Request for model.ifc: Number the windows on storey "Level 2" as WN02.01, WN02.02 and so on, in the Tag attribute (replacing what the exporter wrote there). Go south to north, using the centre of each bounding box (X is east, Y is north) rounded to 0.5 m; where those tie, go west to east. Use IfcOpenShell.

First a look at what the model holds.

```python
import ifcopenshell
import ifcopenshell.util.element
import ifcopenshell.util.placement

model = ifcopenshell.open("model.ifc")
print(model.schema)
storey = next(s for s in model.by_type("IfcBuildingStorey") if s.Name == "Level 2")
windows = [e for e in ifcopenshell.util.element.get_decomposition(storey) if e.is_a("IfcWindow")]
for e in sorted(windows, key=lambda e: e.id()):
    origin = ifcopenshell.util.placement.get_local_placement(e.ObjectPlacement)[:3, 3]
    print(e.id(), e.Tag, e.Name, origin.round(2) + 0.0, sep=" | ")
```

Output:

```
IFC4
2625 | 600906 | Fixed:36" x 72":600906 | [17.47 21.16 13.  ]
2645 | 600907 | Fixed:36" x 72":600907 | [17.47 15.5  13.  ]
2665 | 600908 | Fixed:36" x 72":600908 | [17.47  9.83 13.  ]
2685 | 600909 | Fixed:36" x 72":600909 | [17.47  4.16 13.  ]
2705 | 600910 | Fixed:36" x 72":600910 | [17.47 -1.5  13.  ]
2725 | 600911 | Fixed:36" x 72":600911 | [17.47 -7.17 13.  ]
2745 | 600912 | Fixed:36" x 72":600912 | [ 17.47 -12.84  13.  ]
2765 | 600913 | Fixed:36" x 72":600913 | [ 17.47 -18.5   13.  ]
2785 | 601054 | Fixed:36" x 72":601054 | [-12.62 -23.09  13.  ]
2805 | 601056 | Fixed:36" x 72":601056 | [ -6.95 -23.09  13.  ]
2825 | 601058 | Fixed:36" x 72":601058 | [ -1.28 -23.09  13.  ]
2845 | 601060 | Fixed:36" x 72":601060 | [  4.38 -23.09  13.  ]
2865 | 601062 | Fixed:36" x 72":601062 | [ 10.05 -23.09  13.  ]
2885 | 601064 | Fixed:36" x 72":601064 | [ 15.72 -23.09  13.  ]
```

```python
import ifcopenshell
import ifcopenshell.geom
import ifcopenshell.util.element
import ifcopenshell.util.shape

model = ifcopenshell.open("model.ifc")
settings = ifcopenshell.geom.settings()
settings.set("use-world-coords", True)


def centre(element):
    shape = ifcopenshell.geom.create_shape(settings, element)
    return ifcopenshell.util.shape.get_bbox_centroid(shape.geometry)


storey = next(s for s in model.by_type("IfcBuildingStorey") if s.Name == "Level 2")
windows = [e for e in ifcopenshell.util.element.get_decomposition(storey) if e.is_a("IfcWindow")]

# Insertion points can sit at a corner or the storey origin, so sort by the geometry (in metres).
centres = {e: centre(e) for e in windows}
windows.sort(key=lambda e: (round(centres[e][1] / 0.5), centres[e][0]))

for i, e in enumerate(windows, start=1):
    number = f"WN02.{i:02d}"
    e.Tag = number
    print(e.id(), number)

model.write("model_updated.ifc")
```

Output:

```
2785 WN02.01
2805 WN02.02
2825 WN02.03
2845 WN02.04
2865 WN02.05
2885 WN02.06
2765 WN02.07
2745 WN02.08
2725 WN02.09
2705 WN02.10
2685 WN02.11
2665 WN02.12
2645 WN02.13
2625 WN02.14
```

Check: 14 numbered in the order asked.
